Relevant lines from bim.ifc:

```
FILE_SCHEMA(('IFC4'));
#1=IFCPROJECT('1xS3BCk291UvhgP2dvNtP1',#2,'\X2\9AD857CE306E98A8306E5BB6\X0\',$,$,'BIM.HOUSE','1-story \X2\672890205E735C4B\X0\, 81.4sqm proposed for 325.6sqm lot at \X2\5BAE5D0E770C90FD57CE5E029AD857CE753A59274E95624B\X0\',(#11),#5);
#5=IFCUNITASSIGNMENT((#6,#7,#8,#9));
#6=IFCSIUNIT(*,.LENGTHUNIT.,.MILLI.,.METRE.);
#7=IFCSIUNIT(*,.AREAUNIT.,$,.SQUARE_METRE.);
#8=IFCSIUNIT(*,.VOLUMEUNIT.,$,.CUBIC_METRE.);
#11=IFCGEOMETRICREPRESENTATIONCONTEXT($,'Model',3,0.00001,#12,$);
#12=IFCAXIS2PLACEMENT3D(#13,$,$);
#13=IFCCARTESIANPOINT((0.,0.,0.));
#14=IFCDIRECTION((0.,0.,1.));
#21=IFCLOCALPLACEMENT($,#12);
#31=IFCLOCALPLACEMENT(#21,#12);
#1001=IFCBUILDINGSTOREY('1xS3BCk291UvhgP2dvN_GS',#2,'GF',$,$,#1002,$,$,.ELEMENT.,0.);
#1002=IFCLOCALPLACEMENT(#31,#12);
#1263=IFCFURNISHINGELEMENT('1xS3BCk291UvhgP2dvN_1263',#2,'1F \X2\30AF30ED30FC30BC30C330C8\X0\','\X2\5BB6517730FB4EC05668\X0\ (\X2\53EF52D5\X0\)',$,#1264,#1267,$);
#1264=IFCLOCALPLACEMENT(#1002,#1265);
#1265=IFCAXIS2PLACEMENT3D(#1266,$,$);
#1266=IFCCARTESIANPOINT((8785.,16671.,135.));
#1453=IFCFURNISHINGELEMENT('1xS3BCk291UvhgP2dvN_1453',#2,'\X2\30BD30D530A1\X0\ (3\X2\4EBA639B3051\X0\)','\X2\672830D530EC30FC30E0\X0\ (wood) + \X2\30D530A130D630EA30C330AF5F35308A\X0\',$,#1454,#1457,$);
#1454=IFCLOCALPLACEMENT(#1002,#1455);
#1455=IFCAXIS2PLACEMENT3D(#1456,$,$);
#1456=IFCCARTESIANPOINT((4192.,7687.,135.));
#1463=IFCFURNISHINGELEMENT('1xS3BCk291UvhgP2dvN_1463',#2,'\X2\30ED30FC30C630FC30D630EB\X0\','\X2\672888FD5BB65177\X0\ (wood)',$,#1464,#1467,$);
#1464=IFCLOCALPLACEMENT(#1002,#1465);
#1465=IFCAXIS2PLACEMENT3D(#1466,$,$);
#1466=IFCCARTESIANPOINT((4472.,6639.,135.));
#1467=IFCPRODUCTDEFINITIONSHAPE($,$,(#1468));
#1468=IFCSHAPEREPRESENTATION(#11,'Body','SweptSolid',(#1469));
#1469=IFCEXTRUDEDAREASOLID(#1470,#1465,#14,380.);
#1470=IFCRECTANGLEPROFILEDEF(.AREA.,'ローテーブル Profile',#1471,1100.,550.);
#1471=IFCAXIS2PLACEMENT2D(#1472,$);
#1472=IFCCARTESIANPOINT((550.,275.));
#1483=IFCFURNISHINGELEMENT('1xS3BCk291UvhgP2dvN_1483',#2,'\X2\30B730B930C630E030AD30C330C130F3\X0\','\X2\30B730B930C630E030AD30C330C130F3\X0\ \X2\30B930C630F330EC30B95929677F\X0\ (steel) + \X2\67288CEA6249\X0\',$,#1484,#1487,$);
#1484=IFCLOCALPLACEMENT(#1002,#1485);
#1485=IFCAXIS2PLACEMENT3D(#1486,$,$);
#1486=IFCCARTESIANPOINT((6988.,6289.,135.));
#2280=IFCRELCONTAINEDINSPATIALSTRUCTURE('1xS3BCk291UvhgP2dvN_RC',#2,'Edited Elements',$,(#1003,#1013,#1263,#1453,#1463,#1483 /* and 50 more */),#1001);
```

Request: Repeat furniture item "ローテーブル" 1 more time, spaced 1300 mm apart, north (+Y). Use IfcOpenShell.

```python
import numpy as np
import ifcopenshell
import ifcopenshell.api.geometry
import ifcopenshell.api.root
import ifcopenshell.util.element
import ifcopenshell.util.placement

model = ifcopenshell.open("bim.ifc")


def reuse_history(source, copy):
    """copy_class also copies each property set's owner history, people and application; keep the originals."""
    for rel in copy.IsDefinedBy:
        if rel.is_a("IfcRelDefinesByProperties") and (history := rel.RelatingPropertyDefinition.OwnerHistory):
            rel.RelatingPropertyDefinition.OwnerHistory = source.OwnerHistory
            ifcopenshell.util.element.remove_deep2(model, history)


source = model.by_guid("1xS3BCk291UvhgP2dvN_1463")
base = ifcopenshell.util.placement.get_local_placement(source.ObjectPlacement)
step = np.array([0.0, 1.0, 0.0]) * 1300.0

for i in range(1, 2):
    copy = ifcopenshell.api.root.copy_class(model, product=source)
    copy.Representation = ifcopenshell.util.element.copy_deep(
        model, source.Representation, exclude=["IfcGeometricRepresentationContext", "IfcRepresentationMap"]
    )
    reuse_history(source, copy)
    matrix = base.copy()
    matrix[:3, 3] += i * step
    print("added at", matrix[:3, 3].round(3) + 0.0)
    ifcopenshell.api.geometry.edit_object_placement(model, product=copy, matrix=matrix, is_si=False)

model.write("bim-out.ifc")
```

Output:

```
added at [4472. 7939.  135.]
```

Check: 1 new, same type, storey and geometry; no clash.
